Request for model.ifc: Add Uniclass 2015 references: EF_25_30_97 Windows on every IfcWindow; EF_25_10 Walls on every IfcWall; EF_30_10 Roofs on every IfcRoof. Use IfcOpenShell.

First a look at what the model holds.

```python
import ifcopenshell

model = ifcopenshell.open("model.ifc")
print(model.schema)
print("classifications:", [c.Name for c in model.by_type("IfcClassification")])
for ifc_class in ("IfcDoor", "IfcRoof", "IfcStair", "IfcWall", "IfcWindow"):
    print(ifc_class, len(model.by_type(ifc_class)))
```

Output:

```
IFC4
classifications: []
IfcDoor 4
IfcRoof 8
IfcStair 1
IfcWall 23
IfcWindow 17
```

```python
import ifcopenshell
import ifcopenshell.api.classification

model = ifcopenshell.open("model.ifc")

system = ifcopenshell.api.classification.add_classification(model, classification="Uniclass 2015")

codes = {
    "IfcWindow": ("EF_25_30_97", "Windows"),
    "IfcWall": ("EF_25_10", "Walls"),
    "IfcRoof": ("EF_30_10", "Roofs"),
}
for ifc_class, (code, name) in codes.items():
    products = model.by_type(ifc_class)
    ifcopenshell.api.classification.add_reference(
        model, products=products, classification=system, identification=code, name=name
    )
    print(code, len(products))

model.write("model_rev.ifc")
```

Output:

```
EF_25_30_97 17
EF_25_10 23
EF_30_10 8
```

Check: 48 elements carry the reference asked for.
